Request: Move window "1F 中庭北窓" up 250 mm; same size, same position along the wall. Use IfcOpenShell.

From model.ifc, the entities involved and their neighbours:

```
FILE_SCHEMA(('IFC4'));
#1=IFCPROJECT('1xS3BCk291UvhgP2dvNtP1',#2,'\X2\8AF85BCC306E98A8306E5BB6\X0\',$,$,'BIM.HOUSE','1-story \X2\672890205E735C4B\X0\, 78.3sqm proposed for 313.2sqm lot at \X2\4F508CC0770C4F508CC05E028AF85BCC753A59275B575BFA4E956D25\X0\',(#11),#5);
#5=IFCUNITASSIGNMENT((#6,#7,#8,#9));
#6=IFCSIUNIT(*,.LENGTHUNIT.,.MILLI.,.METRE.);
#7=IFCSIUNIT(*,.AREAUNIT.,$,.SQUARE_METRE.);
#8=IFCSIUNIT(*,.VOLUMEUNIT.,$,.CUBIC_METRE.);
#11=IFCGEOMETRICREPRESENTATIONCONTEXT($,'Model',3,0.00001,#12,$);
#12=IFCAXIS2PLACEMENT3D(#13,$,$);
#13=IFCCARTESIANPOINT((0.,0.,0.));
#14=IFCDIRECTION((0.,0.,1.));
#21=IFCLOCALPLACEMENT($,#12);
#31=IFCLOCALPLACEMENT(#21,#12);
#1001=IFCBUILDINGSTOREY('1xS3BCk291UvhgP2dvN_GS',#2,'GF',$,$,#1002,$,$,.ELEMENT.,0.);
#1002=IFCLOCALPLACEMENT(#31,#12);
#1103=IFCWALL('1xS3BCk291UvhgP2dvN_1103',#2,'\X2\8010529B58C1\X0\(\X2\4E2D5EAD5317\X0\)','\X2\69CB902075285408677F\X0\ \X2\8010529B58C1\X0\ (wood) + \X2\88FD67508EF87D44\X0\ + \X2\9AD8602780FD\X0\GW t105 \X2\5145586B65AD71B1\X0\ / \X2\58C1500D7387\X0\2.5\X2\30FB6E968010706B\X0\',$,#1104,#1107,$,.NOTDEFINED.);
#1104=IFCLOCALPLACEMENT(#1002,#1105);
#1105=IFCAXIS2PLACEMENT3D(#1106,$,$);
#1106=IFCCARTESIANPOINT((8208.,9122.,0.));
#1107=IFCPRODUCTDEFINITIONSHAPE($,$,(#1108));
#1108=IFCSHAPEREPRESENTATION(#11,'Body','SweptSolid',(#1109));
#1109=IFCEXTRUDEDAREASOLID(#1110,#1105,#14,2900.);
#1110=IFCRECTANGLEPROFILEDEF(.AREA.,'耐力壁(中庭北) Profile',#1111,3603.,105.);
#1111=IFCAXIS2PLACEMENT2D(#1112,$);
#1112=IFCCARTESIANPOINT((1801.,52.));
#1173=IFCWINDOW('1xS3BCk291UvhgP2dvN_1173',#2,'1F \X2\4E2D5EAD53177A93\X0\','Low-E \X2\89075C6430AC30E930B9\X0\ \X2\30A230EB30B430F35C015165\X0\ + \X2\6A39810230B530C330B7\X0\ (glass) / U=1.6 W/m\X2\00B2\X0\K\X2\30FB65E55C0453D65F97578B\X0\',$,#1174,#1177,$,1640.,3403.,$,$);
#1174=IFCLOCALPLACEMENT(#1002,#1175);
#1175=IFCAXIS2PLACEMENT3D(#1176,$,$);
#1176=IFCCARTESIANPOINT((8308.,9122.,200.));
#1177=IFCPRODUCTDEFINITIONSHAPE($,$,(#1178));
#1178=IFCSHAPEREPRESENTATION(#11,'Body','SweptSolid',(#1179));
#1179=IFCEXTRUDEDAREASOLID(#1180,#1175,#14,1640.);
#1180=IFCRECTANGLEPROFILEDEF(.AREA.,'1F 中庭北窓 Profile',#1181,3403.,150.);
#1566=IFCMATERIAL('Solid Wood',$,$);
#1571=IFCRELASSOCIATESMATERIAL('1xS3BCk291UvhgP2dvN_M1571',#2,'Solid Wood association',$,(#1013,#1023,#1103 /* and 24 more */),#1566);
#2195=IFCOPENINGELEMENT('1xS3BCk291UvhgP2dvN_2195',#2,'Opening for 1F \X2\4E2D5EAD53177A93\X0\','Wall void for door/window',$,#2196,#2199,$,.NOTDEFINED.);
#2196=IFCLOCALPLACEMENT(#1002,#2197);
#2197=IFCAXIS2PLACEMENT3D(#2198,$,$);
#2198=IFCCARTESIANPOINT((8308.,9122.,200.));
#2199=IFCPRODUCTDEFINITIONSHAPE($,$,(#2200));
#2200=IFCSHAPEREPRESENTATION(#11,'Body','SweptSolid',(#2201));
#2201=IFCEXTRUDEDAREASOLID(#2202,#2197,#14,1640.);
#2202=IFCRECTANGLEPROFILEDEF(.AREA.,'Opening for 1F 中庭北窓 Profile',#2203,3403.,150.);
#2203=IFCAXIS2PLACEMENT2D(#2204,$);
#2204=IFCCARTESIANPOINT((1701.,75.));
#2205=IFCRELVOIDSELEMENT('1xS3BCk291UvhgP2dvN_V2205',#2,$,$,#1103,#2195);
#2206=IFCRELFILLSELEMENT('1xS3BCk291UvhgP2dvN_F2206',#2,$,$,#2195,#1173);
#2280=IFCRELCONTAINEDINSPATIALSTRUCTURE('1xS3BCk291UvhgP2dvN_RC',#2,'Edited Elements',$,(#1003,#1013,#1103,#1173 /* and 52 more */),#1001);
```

```python
import numpy as np
import ifcopenshell
import ifcopenshell.api.geometry
import ifcopenshell.util.placement
import ifcopenshell.util.unit

model = ifcopenshell.open("model.ifc")
unit_scale = ifcopenshell.util.unit.calculate_unit_scale(model)

window = model.by_guid("1xS3BCk291UvhgP2dvN_1173")
opening = window.FillsVoids[0].RelatingOpeningElement
dz = 0.25 / unit_scale

shift = np.array([0.0, 0.0, dz])
# The window is not placed relative to its opening, so move both.
for product in (opening, window):
    matrix = ifcopenshell.util.placement.get_local_placement(product.ObjectPlacement)
    matrix[:3, 3] += shift
    ifcopenshell.api.geometry.edit_object_placement(model, product=product, matrix=matrix, is_si=False)

print(f"moved by {dz * unit_scale:+.3f} m")

model.write("model_edited.ifc")
```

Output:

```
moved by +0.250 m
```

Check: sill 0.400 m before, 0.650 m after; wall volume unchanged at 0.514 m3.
